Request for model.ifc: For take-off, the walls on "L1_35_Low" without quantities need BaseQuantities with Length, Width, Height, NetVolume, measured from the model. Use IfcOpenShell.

First a look at what the model holds.

```python
import ifcopenshell
import ifcopenshell.util.element
import ifcopenshell.util.unit

model = ifcopenshell.open("model.ifc")
print(model.schema)
for unit_type in ("LENGTHUNIT", "AREAUNIT", "VOLUMEUNIT"):
    print(unit_type, ifcopenshell.util.unit.calculate_unit_scale(model, unit_type))
storey = next(s for s in model.by_type("IfcBuildingStorey") if s.Name == "L1_35_Low")
walls = [e for e in ifcopenshell.util.element.get_decomposition(storey) if e.is_a("IfcWall")]
for e in sorted(walls, key=lambda e: e.id()):
    print(e.id(), e.is_a(), e.Name, list(ifcopenshell.util.element.get_psets(e, qtos_only=True)), sep=" | ")
```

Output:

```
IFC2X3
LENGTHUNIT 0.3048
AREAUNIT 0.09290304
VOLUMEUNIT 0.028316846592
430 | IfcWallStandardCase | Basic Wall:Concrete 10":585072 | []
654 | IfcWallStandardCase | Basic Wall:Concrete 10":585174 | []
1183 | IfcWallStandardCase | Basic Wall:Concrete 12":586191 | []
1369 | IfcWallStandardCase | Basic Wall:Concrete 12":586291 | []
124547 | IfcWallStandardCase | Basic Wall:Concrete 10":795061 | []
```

```python
import ifcopenshell
import ifcopenshell.api.pset
import ifcopenshell.geom
import ifcopenshell.util.element
import ifcopenshell.util.shape
import ifcopenshell.util.unit

model = ifcopenshell.open("model.ifc")
unit_scale = ifcopenshell.util.unit.calculate_unit_scale(model)
volume_scale = ifcopenshell.util.unit.calculate_unit_scale(model, "VOLUMEUNIT")
settings = ifcopenshell.geom.settings()

storey = next(s for s in model.by_type("IfcBuildingStorey") if s.Name == "L1_35_Low")
walls = [e for e in ifcopenshell.util.element.get_decomposition(storey) if e.is_a("IfcWall")]

for e in sorted(walls, key=lambda e: e.id()):
    if ifcopenshell.util.element.get_psets(e, qtos_only=True, should_inherit=False):
        continue
    # Geometry comes back in metres, in the element's own axes.
    shape = ifcopenshell.geom.create_shape(settings, e)
    values = {
        "Length": ifcopenshell.util.shape.get_x(shape.geometry) / unit_scale,
        "Width": ifcopenshell.util.shape.get_y(shape.geometry) / unit_scale,
        "Height": ifcopenshell.util.shape.get_z(shape.geometry) / unit_scale,
        "NetVolume": ifcopenshell.util.shape.get_volume(shape.geometry) / volume_scale,
    }
    qto = ifcopenshell.api.pset.add_qto(model, product=e, name="BaseQuantities")
    ifcopenshell.api.pset.edit_qto(model, qto=qto, properties=values)
    print(e.id(), {k: round(v, 3) for k, v in values.items()})

model.write("model_edited.ifc")
```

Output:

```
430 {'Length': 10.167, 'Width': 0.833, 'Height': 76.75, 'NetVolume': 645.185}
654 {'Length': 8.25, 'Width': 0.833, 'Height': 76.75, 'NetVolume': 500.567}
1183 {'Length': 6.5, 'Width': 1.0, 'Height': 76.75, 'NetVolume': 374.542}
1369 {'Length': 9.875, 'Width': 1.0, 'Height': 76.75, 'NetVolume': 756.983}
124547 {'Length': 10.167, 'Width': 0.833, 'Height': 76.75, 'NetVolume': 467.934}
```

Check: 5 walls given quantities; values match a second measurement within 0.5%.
